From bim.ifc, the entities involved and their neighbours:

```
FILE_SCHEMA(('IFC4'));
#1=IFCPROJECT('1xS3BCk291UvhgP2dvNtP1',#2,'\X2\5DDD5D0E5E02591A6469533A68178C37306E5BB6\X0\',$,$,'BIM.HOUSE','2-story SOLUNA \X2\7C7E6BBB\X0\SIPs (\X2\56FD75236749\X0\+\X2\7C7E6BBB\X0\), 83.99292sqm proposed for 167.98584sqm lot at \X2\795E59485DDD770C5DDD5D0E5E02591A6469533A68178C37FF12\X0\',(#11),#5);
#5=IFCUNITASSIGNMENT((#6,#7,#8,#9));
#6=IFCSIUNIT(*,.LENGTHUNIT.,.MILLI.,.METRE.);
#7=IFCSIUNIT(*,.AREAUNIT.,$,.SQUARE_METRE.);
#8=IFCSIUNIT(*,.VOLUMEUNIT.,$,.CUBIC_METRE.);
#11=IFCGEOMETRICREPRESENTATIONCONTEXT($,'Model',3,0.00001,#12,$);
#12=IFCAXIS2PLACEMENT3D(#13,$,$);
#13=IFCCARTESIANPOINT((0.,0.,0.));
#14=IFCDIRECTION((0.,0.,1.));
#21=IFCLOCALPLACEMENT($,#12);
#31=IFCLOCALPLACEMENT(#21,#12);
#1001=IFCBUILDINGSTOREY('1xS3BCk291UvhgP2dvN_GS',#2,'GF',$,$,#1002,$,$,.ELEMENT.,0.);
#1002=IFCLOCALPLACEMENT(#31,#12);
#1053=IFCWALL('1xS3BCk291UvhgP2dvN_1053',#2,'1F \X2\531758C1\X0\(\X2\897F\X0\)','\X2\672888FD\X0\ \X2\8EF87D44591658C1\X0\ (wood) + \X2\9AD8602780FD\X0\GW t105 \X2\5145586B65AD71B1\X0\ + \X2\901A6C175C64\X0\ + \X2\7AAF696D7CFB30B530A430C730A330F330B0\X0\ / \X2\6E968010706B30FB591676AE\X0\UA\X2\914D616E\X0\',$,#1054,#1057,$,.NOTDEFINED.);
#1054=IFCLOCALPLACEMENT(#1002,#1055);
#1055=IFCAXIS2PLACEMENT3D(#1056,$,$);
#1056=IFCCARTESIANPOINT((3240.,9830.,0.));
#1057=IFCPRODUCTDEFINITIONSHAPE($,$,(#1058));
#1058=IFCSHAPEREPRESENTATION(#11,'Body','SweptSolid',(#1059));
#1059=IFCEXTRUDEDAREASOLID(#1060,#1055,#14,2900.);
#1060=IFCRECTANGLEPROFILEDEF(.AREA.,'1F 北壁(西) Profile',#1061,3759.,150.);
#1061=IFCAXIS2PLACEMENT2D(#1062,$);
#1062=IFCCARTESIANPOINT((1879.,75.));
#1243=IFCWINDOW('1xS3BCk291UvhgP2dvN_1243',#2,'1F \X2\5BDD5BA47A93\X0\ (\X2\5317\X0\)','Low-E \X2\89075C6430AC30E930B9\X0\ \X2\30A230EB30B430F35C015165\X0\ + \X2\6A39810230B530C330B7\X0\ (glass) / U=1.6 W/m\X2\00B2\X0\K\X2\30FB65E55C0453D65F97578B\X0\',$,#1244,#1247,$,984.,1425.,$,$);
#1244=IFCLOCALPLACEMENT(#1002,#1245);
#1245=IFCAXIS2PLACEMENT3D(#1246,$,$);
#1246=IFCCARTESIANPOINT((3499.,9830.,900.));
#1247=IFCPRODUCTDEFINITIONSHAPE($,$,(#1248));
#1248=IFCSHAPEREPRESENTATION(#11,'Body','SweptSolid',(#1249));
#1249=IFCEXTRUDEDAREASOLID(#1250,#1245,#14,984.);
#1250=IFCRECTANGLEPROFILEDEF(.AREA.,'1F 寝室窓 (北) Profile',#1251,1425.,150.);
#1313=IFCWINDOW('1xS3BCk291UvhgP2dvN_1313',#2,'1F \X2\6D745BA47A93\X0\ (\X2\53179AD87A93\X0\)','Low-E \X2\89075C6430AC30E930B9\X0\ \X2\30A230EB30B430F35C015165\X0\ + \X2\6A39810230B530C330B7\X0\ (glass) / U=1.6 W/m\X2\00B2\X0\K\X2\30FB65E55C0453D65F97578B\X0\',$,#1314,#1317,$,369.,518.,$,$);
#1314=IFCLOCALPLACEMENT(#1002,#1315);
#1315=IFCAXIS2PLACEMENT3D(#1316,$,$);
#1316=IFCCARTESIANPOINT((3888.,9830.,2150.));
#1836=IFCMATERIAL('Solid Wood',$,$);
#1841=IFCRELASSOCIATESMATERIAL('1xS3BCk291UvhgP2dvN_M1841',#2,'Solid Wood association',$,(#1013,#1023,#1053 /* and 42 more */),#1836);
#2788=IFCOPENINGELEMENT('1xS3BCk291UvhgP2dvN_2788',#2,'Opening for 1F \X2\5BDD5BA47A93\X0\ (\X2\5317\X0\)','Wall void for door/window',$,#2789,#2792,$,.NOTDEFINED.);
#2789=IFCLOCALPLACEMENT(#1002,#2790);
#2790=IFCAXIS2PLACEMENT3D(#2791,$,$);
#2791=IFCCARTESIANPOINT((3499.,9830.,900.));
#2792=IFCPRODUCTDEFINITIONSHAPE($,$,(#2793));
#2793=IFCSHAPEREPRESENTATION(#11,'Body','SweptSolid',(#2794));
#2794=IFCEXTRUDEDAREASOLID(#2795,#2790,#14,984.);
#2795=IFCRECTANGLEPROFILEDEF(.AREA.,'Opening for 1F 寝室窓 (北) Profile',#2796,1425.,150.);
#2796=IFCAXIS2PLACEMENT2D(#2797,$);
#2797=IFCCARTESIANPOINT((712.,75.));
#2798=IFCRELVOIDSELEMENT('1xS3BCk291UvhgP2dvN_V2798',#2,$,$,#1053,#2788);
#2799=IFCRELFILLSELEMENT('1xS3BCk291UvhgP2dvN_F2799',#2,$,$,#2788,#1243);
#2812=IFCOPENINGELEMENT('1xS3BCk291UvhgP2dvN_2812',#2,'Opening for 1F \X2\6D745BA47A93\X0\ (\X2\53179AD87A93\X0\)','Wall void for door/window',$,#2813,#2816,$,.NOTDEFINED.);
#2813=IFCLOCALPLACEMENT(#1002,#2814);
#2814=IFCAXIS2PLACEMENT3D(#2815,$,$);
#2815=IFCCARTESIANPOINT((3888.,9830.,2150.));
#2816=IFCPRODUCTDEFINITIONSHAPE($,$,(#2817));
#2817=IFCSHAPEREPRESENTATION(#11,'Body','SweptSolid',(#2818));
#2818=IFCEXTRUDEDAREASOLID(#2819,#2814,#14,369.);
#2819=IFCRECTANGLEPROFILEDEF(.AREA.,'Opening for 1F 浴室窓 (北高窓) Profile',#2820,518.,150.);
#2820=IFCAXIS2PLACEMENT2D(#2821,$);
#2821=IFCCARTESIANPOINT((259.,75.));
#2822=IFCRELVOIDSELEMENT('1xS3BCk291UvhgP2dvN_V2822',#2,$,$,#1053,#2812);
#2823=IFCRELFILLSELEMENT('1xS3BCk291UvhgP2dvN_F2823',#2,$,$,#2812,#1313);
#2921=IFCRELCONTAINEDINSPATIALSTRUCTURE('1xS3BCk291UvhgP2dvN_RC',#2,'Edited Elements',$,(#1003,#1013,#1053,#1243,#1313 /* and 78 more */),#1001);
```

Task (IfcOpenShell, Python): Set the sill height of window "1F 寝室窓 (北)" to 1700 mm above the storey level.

```python
import numpy as np
import ifcopenshell
import ifcopenshell.api.geometry
import ifcopenshell.geom
import ifcopenshell.util.element
import ifcopenshell.util.placement
import ifcopenshell.util.shape
import ifcopenshell.util.unit

model = ifcopenshell.open("bim.ifc")
unit_scale = ifcopenshell.util.unit.calculate_unit_scale(model)

window = model.by_guid("1xS3BCk291UvhgP2dvN_1243")
opening = window.FillsVoids[0].RelatingOpeningElement
storey = ifcopenshell.util.element.get_container(window, ifc_class="IfcBuildingStorey")
level = ifcopenshell.util.placement.get_local_placement(storey.ObjectPlacement)[2, 3]

# The opening's origin need not be at the sill, so measure its lowest point.
shape = ifcopenshell.geom.create_shape(ifcopenshell.geom.settings(), opening)
bottom = ifcopenshell.util.shape.get_shape_bottom_elevation(shape, shape.geometry) / unit_scale
dz = level + 1.7 / unit_scale - bottom

shift = np.array([0.0, 0.0, dz])
# The window is not placed relative to its opening, so move both.
for product in (opening, window):
    matrix = ifcopenshell.util.placement.get_local_placement(product.ObjectPlacement)
    matrix[:3, 3] += shift
    ifcopenshell.api.geometry.edit_object_placement(model, product=product, matrix=matrix, is_si=False)

print(f"moved by {dz * unit_scale:+.3f} m")

model.write("bim_edited.ifc")
```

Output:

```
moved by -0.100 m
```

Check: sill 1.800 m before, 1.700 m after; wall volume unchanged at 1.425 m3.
